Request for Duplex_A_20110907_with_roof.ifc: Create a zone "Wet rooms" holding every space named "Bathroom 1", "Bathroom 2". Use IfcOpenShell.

First a look at what the model holds.

```python
import ifcopenshell

model = ifcopenshell.open("Duplex_A_20110907_with_roof.ifc")
print(model.schema)
seen = {}
for space in model.by_type("IfcSpace"):
    seen[space.LongName] = seen.get(space.LongName, 0) + 1
for name, count in sorted(seen.items(), key=str):
    print(count, "x", name)
print("zones:", [z.Name for z in model.by_type("IfcZone")][:20])
```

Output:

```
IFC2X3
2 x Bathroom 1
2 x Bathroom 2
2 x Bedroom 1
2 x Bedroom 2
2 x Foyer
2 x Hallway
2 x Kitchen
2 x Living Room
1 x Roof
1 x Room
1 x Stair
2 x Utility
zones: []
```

```python
import ifcopenshell
import ifcopenshell.api.group
import ifcopenshell.api.root

model = ifcopenshell.open("Duplex_A_20110907_with_roof.ifc")

names = {"Bathroom 1", "Bathroom 2"}
spaces = [s for s in model.by_type("IfcSpace") if s.LongName in names]

zone = ifcopenshell.api.root.create_entity(model, ifc_class="IfcZone", name="Wet rooms")
ifcopenshell.api.group.assign_group(model, products=spaces, group=zone)
print(len(spaces), "spaces in", zone.Name)

model.write("Duplex_A_20110907_with_roof_v2.ifc")
```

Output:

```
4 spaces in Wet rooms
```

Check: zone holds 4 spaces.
